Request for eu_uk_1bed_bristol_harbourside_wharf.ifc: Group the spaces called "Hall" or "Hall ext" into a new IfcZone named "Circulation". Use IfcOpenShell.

First a look at what the model holds.

```python
import ifcopenshell

model = ifcopenshell.open("eu_uk_1bed_bristol_harbourside_wharf.ifc")
print(model.schema)
seen = {}
for space in model.by_type("IfcSpace"):
    seen[space.LongName] = seen.get(space.LongName, 0) + 1
for name, count in sorted(seen.items(), key=str):
    print(count, "x", name)
print("zones:", [z.Name for z in model.by_type("IfcZone")][:20])
```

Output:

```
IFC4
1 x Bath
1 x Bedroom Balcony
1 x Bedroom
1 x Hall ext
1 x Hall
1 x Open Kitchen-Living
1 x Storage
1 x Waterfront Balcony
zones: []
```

```python
import ifcopenshell
import ifcopenshell.api.group
import ifcopenshell.api.root

model = ifcopenshell.open("eu_uk_1bed_bristol_harbourside_wharf.ifc")

names = {"Hall", "Hall ext"}
spaces = [s for s in model.by_type("IfcSpace") if s.LongName in names]

zone = ifcopenshell.api.root.create_entity(model, ifc_class="IfcZone", name="Circulation")
ifcopenshell.api.group.assign_group(model, products=spaces, group=zone)
print(len(spaces), "spaces in", zone.Name)

model.write("eu_uk_1bed_bristol_harbourside_wharf_v2.ifc")
```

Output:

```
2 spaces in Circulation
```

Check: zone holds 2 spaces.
